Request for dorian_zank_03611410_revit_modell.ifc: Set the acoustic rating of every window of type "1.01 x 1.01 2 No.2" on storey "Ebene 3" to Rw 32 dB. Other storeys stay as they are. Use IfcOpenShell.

First a look at what the model holds.

```python
import ifcopenshell
import ifcopenshell.util.element

model = ifcopenshell.open("dorian_zank_03611410_revit_modell.ifc")
print(model.schema)
storey = next(s for s in model.by_type("IfcBuildingStorey") if s.Name == "Ebene 3")
windows = [e for e in ifcopenshell.util.element.get_decomposition(storey) if e.is_a("IfcWindow")]
seen = {}
for e in windows:
    element_type = ifcopenshell.util.element.get_type(e)
    key = (element_type.Name if element_type != e and element_type else None, ifcopenshell.util.element.get_pset(e, "Pset_WindowCommon", "AcousticRating"))
    seen[key] = seen.get(key, 0) + 1
for (name, value), count in sorted(seen.items(), key=str):
    print(count, "x", name, "|", value)
```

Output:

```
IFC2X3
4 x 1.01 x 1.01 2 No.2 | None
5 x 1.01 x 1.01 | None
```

```python
import ifcopenshell
import ifcopenshell.api.pset
import ifcopenshell.util.element

model = ifcopenshell.open("dorian_zank_03611410_revit_modell.ifc")

storey = next(s for s in model.by_type("IfcBuildingStorey") if s.Name == "Ebene 3")
windows = [e for e in ifcopenshell.util.element.get_decomposition(storey) if e.is_a("IfcWindow")]

count = 0
for e in windows:
    element_type = ifcopenshell.util.element.get_type(e)
    if element_type in (None, e) or element_type.Name != "1.01 x 1.01 2 No.2":
        continue
    # add_pset returns the element's existing set when there is one.
    pset = ifcopenshell.api.pset.add_pset(model, product=e, name="Pset_WindowCommon")
    ifcopenshell.api.pset.edit_pset(model, pset=pset, properties={"AcousticRating": "Rw 32 dB"})
    count += 1

print(count, "windows updated")

model.write("dorian_zank_03611410_revit_modell_v2.ifc")
```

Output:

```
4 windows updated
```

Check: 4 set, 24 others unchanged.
